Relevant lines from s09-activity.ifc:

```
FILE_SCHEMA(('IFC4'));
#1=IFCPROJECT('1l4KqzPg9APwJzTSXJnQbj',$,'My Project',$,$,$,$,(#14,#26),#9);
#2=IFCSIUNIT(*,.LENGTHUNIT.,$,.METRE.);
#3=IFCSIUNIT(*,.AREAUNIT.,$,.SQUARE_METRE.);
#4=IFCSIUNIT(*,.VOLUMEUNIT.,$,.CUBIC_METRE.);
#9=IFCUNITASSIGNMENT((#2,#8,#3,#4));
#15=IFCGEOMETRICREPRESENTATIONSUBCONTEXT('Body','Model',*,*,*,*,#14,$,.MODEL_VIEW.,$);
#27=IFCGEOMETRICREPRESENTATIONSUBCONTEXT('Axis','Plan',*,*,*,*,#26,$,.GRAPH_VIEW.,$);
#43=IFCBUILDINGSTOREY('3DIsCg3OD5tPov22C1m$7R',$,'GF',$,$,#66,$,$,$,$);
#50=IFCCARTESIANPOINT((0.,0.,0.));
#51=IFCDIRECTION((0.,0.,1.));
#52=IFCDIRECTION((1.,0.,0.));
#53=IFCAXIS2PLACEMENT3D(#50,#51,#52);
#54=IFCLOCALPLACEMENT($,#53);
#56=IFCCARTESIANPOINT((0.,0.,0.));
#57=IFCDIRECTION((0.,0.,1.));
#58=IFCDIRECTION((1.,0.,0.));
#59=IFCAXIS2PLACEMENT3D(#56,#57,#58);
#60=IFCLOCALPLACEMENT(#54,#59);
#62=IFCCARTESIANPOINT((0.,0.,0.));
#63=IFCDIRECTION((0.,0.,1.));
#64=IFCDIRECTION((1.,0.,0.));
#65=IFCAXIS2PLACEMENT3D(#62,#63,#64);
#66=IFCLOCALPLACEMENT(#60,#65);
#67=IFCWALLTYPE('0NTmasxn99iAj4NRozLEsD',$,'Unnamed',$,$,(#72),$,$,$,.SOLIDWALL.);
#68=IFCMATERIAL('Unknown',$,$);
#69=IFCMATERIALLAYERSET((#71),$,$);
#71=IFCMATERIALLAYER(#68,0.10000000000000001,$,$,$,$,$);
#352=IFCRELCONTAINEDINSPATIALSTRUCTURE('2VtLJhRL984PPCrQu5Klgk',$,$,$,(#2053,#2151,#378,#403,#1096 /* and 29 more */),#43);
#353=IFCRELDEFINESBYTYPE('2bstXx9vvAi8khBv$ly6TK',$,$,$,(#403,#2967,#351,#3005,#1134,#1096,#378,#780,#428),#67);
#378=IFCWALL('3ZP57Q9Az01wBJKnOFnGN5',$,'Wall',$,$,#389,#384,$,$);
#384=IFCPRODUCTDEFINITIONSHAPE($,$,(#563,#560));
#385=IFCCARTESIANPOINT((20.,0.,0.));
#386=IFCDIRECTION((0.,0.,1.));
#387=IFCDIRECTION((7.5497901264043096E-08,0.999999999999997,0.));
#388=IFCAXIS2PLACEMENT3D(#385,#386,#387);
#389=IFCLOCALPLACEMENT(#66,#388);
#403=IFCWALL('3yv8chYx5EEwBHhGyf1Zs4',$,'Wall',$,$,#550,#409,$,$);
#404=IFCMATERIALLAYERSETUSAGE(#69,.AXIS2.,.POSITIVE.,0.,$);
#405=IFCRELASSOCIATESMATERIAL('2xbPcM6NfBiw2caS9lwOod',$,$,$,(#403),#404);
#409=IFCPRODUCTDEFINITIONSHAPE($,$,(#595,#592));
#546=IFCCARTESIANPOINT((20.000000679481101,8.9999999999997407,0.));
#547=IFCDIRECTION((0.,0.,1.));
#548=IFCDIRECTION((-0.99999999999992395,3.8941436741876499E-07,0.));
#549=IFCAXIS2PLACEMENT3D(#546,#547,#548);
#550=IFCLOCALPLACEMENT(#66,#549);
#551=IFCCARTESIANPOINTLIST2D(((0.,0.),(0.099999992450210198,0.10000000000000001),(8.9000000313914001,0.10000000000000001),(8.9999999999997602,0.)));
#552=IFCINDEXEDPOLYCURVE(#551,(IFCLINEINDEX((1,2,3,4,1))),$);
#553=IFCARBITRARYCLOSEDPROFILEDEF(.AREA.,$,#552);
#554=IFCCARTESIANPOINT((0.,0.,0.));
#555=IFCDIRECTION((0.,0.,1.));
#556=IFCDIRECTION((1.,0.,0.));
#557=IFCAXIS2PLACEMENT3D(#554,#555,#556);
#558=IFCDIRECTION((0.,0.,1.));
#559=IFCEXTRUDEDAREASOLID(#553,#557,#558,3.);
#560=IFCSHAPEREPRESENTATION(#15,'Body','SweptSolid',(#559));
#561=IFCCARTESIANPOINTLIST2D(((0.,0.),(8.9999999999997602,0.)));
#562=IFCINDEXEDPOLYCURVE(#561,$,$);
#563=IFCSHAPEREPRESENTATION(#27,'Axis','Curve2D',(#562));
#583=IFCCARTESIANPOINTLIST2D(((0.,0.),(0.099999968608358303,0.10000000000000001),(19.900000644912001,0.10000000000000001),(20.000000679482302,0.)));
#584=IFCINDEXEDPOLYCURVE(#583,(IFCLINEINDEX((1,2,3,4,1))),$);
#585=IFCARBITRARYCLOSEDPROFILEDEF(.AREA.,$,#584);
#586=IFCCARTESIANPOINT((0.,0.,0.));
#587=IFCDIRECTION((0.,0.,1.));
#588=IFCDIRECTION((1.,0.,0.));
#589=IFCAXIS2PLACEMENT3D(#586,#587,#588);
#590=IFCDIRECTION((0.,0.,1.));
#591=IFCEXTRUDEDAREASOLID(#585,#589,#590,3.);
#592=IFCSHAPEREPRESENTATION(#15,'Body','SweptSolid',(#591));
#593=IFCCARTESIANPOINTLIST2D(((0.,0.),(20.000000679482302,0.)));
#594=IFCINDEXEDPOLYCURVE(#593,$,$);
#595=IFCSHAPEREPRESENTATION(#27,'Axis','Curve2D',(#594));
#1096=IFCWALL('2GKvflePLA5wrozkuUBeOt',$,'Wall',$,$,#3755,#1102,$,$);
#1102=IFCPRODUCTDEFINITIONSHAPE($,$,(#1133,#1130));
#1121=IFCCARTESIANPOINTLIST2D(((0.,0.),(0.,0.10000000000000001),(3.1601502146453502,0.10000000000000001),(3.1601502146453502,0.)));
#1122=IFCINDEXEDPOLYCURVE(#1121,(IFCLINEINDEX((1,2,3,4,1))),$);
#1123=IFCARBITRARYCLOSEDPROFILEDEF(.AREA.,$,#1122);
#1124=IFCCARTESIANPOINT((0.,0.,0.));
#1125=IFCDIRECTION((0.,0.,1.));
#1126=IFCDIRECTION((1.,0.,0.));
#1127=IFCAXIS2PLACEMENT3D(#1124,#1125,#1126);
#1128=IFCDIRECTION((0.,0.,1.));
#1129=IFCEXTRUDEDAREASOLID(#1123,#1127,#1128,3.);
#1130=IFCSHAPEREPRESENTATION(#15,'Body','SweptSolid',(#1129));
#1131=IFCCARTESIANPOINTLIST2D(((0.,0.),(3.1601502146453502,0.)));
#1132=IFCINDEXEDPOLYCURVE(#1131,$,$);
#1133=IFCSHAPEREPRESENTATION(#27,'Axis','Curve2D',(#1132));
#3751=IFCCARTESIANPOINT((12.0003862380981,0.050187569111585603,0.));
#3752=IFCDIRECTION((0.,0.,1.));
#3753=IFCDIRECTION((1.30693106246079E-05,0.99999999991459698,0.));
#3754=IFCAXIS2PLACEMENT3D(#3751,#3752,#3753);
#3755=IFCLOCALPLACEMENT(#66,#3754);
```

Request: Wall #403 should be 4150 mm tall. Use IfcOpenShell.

```python
import ifcopenshell
import ifcopenshell.geom
import ifcopenshell.util.representation
import ifcopenshell.util.shape
import ifcopenshell.util.unit

model = ifcopenshell.open("s09-activity.ifc")
unit_scale = ifcopenshell.util.unit.calculate_unit_scale(model)
settings = ifcopenshell.geom.settings()


def volume(element):
    """Net volume in cubic metres, openings subtracted."""
    shape = ifcopenshell.geom.create_shape(settings, element)
    return ifcopenshell.util.shape.get_volume(shape.geometry)


wall = model.by_guid("3yv8chYx5EEwBHhGyf1Zs4")
before = volume(wall)

body = ifcopenshell.util.representation.get_representation(wall, "Model", "Body")
solid = body.Items[0]
old_height = solid.Depth
solid.Depth = 4.15 / unit_scale
after = volume(wall)

print(f"height {old_height:g} -> {solid.Depth:g}, volume {before:.3f} -> {after:.3f} m3")

model.write("s09-activity-out.ifc")
```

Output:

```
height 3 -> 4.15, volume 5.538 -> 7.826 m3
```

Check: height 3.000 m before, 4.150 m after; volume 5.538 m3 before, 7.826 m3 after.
